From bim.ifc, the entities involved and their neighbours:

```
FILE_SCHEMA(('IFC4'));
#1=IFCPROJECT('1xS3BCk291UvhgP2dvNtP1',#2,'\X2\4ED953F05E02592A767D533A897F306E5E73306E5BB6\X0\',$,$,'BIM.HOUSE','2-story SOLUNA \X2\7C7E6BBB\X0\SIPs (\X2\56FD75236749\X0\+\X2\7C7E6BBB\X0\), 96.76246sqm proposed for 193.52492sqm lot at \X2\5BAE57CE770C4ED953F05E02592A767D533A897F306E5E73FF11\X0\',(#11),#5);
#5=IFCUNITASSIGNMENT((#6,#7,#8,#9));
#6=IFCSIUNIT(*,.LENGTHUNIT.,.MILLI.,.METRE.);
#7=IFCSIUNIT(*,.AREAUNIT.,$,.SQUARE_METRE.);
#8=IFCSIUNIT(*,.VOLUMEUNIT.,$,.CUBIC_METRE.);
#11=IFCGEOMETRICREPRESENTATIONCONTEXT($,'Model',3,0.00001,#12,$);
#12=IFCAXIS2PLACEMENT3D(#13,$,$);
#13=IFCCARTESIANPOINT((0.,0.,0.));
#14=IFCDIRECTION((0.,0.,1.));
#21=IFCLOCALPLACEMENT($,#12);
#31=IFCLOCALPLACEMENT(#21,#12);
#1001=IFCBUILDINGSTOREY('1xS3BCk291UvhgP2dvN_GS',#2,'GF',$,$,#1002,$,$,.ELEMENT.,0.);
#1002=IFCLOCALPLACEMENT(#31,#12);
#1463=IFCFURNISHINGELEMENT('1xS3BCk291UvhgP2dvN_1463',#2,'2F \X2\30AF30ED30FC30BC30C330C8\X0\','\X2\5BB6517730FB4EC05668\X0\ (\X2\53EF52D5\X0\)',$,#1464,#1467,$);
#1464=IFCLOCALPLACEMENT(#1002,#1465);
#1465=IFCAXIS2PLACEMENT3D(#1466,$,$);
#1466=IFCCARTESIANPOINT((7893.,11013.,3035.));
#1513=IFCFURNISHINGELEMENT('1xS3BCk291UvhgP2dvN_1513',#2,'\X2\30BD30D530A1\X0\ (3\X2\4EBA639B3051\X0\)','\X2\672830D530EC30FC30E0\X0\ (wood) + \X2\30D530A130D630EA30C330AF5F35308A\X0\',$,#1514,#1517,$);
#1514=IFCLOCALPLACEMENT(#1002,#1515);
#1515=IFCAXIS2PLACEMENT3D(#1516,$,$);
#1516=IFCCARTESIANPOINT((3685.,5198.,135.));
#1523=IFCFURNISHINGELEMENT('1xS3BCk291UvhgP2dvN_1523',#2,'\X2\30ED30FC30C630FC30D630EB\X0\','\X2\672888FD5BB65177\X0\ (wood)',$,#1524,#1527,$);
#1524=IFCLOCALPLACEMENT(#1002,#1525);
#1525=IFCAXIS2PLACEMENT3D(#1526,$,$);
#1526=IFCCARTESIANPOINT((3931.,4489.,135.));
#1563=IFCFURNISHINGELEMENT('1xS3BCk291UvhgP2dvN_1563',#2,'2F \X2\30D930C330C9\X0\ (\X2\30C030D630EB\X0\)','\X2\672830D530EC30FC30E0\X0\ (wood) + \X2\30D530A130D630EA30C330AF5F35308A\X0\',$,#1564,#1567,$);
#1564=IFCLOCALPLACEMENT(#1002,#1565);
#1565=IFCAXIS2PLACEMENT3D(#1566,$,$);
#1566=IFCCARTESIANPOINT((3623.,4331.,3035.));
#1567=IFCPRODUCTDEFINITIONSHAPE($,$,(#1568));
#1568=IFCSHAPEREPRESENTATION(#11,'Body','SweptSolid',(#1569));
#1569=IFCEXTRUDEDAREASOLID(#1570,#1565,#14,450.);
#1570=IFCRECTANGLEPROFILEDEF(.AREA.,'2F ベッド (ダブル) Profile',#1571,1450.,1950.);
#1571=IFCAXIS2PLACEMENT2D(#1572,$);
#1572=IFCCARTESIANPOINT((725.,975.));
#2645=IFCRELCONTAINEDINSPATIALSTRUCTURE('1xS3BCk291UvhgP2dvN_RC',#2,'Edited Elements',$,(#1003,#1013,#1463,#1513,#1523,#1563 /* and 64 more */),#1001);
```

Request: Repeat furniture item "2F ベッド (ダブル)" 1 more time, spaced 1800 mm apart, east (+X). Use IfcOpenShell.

```python
import numpy as np
import ifcopenshell
import ifcopenshell.api.geometry
import ifcopenshell.api.root
import ifcopenshell.util.element
import ifcopenshell.util.placement

model = ifcopenshell.open("bim.ifc")


def reuse_history(source, copy):
    """copy_class also copies each property set's owner history, people and application; keep the originals."""
    for rel in copy.IsDefinedBy:
        if rel.is_a("IfcRelDefinesByProperties") and (history := rel.RelatingPropertyDefinition.OwnerHistory):
            rel.RelatingPropertyDefinition.OwnerHistory = source.OwnerHistory
            ifcopenshell.util.element.remove_deep2(model, history)


source = model.by_guid("1xS3BCk291UvhgP2dvN_1563")
base = ifcopenshell.util.placement.get_local_placement(source.ObjectPlacement)
step = np.array([1.0, 0.0, 0.0]) * 1800.0

for i in range(1, 2):
    copy = ifcopenshell.api.root.copy_class(model, product=source)
    copy.Representation = ifcopenshell.util.element.copy_deep(
        model, source.Representation, exclude=["IfcGeometricRepresentationContext", "IfcRepresentationMap"]
    )
    reuse_history(source, copy)
    matrix = base.copy()
    matrix[:3, 3] += i * step
    print("added at", matrix[:3, 3].round(3) + 0.0)
    ifcopenshell.api.geometry.edit_object_placement(model, product=copy, matrix=matrix, is_si=False)

model.write("bim_updated.ifc")
```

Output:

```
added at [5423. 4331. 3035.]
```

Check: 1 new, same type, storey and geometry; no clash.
